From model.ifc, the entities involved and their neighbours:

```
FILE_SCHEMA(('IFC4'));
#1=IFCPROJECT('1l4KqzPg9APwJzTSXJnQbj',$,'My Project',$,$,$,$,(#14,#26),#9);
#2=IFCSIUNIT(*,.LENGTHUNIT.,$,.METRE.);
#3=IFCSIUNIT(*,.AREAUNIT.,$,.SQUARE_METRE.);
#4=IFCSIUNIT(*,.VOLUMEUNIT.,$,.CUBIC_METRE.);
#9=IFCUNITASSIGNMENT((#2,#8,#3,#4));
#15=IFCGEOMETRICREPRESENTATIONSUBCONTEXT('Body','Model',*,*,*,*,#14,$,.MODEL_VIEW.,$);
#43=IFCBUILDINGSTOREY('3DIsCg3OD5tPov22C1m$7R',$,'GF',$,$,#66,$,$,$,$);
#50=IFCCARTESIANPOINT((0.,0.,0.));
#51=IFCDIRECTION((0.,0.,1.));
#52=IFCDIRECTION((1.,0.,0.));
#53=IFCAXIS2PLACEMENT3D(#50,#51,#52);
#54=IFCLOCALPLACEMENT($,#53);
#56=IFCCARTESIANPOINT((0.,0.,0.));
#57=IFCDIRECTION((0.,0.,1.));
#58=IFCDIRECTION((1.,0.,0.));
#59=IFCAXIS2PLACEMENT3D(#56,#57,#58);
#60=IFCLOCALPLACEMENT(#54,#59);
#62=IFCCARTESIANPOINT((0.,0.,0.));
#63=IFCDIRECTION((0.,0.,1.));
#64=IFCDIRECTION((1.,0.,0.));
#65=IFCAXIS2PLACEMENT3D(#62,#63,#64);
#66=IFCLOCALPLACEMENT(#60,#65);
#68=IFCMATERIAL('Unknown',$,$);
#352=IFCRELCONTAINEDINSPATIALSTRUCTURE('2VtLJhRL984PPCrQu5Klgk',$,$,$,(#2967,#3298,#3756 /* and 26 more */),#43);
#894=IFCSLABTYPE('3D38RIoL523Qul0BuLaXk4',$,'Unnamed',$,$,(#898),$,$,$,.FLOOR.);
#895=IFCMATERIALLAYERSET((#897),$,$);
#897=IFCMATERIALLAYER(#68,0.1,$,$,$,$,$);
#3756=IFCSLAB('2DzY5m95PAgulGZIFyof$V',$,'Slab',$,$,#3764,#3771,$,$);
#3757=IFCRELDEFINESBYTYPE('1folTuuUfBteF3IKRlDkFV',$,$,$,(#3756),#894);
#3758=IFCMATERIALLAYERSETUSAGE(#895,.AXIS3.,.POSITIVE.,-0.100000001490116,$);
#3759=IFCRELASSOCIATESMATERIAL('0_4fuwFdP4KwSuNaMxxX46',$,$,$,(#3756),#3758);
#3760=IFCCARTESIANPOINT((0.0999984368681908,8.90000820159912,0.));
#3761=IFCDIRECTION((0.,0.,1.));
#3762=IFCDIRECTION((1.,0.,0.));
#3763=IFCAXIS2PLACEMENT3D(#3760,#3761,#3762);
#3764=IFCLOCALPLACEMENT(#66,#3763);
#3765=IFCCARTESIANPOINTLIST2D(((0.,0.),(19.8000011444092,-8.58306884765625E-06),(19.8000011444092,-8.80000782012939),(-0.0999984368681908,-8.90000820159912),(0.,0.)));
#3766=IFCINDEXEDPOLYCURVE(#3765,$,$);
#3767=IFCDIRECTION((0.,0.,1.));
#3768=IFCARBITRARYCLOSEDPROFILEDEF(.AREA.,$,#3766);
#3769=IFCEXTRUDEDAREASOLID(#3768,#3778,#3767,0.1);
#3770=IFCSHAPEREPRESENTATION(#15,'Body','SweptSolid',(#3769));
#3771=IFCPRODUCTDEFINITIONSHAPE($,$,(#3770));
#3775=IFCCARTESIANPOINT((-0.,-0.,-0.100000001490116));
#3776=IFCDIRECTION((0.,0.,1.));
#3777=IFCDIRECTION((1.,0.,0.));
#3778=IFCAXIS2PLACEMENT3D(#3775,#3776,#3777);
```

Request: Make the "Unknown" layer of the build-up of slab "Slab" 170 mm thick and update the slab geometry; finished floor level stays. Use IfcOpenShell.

```python
import ifcopenshell
import ifcopenshell.util.element
import ifcopenshell.util.representation
import ifcopenshell.util.unit

model = ifcopenshell.open("model.ifc")
unit_scale = ifcopenshell.util.unit.calculate_unit_scale(model)

layer_set = model.by_id(895)
layer = next(l for l in layer_set.MaterialLayers if l.Material and l.Material.Name == "Unknown")
change = 0.17 / unit_scale - layer.LayerThickness
layer.LayerThickness += change

# Geometry does not follow the layer set by itself.
slabs = [e for e in ifcopenshell.util.element.get_elements_by_material(model, layer_set) if e.is_a("IfcSlab")]
for slab in sorted(slabs, key=lambda e: e.id()):
    body = ifcopenshell.util.representation.get_representation(slab, "Model", "Body")
    solid = body.Items[0]
    old_depth = solid.Depth
    solid.Depth += change
    # Extruded upwards: lower the start of the extrusion so the top stays.
    x, y, z = solid.Position.Location.Coordinates
    solid.Position.Location = model.createIfcCartesianPoint((x, y, z - change))
    print(slab.id(), f"{old_depth:g} -> {solid.Depth:g}")

# The layers are counted up from the underside, which has moved.
for usage in {ifcopenshell.util.element.get_material(slab) for slab in slabs}:
    usage.OffsetFromReferenceLine -= change

model.write("model_updated.ifc")
```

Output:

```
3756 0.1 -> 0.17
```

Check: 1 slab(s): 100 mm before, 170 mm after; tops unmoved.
